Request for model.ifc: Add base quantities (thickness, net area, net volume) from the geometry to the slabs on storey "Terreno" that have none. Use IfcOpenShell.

First a look at what the model holds.

```python
import ifcopenshell
import ifcopenshell.util.element
import ifcopenshell.util.unit

model = ifcopenshell.open("model.ifc")
print(model.schema)
for unit_type in ("LENGTHUNIT", "AREAUNIT", "VOLUMEUNIT"):
    print(unit_type, ifcopenshell.util.unit.calculate_unit_scale(model, unit_type))
storey = next(s for s in model.by_type("IfcBuildingStorey") if s.Name == "Terreno")
slabs = [e for e in ifcopenshell.util.element.get_decomposition(storey) if e.is_a("IfcSlab")]
for e in sorted(slabs, key=lambda e: e.id()):
    print(e.id(), e.is_a(), e.Name, list(ifcopenshell.util.element.get_psets(e, qtos_only=True)), sep=" | ")
```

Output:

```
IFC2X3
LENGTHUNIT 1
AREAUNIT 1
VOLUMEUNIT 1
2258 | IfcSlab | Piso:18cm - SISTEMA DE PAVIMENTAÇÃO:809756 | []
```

```python
import ifcopenshell
import ifcopenshell.api.pset
import ifcopenshell.geom
import ifcopenshell.util.element
import ifcopenshell.util.shape
import ifcopenshell.util.unit

model = ifcopenshell.open("model.ifc")
unit_scale = ifcopenshell.util.unit.calculate_unit_scale(model)
area_scale = ifcopenshell.util.unit.calculate_unit_scale(model, "AREAUNIT")
volume_scale = ifcopenshell.util.unit.calculate_unit_scale(model, "VOLUMEUNIT")
settings = ifcopenshell.geom.settings()

storey = next(s for s in model.by_type("IfcBuildingStorey") if s.Name == "Terreno")
slabs = [e for e in ifcopenshell.util.element.get_decomposition(storey) if e.is_a("IfcSlab")]

for e in sorted(slabs, key=lambda e: e.id()):
    if ifcopenshell.util.element.get_psets(e, qtos_only=True, should_inherit=False):
        continue
    # Geometry comes back in metres, in the element's own axes.
    shape = ifcopenshell.geom.create_shape(settings, e)
    values = {
        "Width": ifcopenshell.util.shape.get_z(shape.geometry) / unit_scale,
        "NetArea": ifcopenshell.util.shape.get_footprint_area(shape.geometry) / area_scale,
        "NetVolume": ifcopenshell.util.shape.get_volume(shape.geometry) / volume_scale,
    }
    qto = ifcopenshell.api.pset.add_qto(model, product=e, name="BaseQuantities")
    ifcopenshell.api.pset.edit_qto(model, qto=qto, properties=values)
    print(e.id(), {k: round(v, 3) for k, v in values.items()})

model.write("model_edited.ifc")
```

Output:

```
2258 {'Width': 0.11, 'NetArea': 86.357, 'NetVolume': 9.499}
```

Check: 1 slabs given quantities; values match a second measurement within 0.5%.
